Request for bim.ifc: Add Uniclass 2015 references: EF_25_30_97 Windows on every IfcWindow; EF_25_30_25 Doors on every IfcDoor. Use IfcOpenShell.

First a look at what the model holds.

```python
import ifcopenshell

model = ifcopenshell.open("bim.ifc")
print(model.schema)
print("classifications:", [c.Name for c in model.by_type("IfcClassification")])
for ifc_class in ("IfcDoor", "IfcRoof", "IfcStair", "IfcWall", "IfcWindow"):
    print(ifc_class, len(model.by_type(ifc_class)))
```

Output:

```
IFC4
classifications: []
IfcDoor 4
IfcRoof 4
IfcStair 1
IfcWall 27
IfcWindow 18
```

```python
import ifcopenshell
import ifcopenshell.api.classification

model = ifcopenshell.open("bim.ifc")

system = ifcopenshell.api.classification.add_classification(model, classification="Uniclass 2015")

codes = {
    "IfcWindow": ("EF_25_30_97", "Windows"),
    "IfcDoor": ("EF_25_30_25", "Doors"),
}
for ifc_class, (code, name) in codes.items():
    products = model.by_type(ifc_class)
    ifcopenshell.api.classification.add_reference(
        model, products=products, classification=system, identification=code, name=name
    )
    print(code, len(products))

model.write("bim_v2.ifc")
```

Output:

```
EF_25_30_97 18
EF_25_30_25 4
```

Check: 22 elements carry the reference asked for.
